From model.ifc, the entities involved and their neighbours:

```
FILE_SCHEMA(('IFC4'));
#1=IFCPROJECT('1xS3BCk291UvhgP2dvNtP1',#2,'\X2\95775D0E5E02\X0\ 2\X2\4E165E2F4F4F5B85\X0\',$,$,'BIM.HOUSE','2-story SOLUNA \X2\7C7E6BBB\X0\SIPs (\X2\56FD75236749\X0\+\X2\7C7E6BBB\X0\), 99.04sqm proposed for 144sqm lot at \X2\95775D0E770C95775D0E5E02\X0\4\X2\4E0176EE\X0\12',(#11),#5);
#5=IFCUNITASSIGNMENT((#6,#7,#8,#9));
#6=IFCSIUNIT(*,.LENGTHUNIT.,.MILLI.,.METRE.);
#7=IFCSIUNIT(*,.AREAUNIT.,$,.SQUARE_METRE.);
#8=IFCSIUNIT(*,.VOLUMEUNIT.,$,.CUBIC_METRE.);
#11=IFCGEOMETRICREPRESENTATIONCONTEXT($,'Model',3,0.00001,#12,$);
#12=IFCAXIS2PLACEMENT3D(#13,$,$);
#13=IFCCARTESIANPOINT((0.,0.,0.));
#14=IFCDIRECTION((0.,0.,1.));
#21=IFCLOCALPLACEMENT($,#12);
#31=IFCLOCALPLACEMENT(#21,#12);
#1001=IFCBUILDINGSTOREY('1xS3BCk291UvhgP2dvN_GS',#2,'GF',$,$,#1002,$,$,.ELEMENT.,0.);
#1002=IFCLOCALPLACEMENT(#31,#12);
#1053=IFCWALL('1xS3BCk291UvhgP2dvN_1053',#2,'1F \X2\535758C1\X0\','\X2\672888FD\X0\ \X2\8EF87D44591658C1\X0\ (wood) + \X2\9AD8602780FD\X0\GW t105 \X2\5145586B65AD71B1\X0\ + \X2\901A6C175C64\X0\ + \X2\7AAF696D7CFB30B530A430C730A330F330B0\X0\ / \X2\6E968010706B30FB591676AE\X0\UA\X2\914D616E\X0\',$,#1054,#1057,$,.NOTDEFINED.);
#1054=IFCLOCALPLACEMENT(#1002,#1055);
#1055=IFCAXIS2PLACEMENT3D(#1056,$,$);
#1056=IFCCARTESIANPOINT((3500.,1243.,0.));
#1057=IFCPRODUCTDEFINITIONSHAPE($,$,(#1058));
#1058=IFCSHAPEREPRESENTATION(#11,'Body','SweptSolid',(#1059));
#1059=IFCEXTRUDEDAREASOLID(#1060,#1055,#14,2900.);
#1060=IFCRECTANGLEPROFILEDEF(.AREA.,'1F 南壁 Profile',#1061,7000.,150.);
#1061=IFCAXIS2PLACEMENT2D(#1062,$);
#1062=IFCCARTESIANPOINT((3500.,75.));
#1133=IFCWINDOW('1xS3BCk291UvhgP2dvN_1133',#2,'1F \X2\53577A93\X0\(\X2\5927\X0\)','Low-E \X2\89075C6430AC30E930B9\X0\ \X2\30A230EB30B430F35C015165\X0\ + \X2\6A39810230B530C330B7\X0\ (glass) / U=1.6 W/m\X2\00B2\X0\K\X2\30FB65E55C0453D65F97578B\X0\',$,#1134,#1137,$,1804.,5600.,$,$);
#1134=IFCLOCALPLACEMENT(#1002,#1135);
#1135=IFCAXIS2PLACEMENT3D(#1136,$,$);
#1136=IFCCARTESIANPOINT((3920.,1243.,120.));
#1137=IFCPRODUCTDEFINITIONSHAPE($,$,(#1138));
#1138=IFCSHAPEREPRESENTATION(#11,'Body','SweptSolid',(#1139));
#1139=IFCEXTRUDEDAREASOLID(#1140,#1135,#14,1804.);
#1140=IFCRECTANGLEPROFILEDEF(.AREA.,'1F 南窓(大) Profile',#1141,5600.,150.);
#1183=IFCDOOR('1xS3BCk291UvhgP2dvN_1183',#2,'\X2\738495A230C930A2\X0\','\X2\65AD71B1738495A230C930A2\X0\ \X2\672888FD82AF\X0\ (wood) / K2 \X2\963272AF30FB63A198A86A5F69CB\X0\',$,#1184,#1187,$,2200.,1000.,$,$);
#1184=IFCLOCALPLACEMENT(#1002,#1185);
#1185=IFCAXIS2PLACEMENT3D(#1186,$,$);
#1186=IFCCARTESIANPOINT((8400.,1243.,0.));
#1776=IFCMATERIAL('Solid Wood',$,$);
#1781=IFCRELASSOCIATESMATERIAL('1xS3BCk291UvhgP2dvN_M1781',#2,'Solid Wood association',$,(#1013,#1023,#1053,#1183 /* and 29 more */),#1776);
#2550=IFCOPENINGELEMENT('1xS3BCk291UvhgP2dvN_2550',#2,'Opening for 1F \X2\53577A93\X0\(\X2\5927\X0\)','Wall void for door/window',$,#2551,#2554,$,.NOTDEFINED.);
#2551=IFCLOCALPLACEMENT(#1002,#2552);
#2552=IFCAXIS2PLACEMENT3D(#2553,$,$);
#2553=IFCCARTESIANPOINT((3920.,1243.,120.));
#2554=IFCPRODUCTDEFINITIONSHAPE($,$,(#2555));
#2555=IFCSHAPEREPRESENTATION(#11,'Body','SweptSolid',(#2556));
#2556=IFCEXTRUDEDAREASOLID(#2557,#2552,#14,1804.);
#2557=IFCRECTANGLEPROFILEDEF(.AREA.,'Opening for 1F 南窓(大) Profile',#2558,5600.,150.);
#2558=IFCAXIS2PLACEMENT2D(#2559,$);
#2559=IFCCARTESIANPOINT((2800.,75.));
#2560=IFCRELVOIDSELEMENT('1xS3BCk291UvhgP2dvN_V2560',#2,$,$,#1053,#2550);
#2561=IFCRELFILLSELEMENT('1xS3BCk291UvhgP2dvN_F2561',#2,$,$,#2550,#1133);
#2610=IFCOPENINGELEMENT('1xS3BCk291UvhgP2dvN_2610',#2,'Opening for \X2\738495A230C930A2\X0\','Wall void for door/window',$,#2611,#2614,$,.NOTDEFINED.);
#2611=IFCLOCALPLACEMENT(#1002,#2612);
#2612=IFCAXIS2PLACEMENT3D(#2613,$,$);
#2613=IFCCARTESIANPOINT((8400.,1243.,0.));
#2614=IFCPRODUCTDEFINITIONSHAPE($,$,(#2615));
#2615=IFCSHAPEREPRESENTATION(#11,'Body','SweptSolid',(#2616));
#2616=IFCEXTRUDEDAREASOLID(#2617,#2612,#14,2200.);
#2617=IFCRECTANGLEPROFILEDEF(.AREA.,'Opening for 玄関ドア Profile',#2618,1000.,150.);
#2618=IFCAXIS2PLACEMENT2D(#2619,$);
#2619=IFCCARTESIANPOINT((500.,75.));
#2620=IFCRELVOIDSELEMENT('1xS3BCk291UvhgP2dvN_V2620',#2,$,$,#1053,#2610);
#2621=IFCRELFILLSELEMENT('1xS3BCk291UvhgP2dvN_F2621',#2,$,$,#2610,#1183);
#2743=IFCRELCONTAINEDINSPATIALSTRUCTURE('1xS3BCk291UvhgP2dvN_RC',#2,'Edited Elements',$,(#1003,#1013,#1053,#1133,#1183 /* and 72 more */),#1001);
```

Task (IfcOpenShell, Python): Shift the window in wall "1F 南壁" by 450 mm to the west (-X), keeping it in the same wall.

```python
import ifcopenshell
import ifcopenshell.api.geometry
import ifcopenshell.util.placement
import ifcopenshell.util.unit

model = ifcopenshell.open("model.ifc")
unit_scale = ifcopenshell.util.unit.calculate_unit_scale(model)

window = model.by_guid("1xS3BCk291UvhgP2dvN_1133")
opening = window.FillsVoids[0].RelatingOpeningElement
wall = opening.VoidsElements[0].RelatingBuildingElement

wall_matrix = ifcopenshell.util.placement.get_local_placement(wall.ObjectPlacement)
shift = wall_matrix[:3, 0] * -0.45 / unit_scale
before = ifcopenshell.util.placement.get_local_placement(window.ObjectPlacement)[:3, 3].copy()

# The window is not placed relative to its opening, so move both.
for product in (opening, window):
    matrix = ifcopenshell.util.placement.get_local_placement(product.ObjectPlacement)
    matrix[:3, 3] += shift
    ifcopenshell.api.geometry.edit_object_placement(model, product=product, matrix=matrix, is_si=False)

after = ifcopenshell.util.placement.get_local_placement(window.ObjectPlacement)[:3, 3]
print("window moved by", (after - before).round(3) + 0.0)

model.write("model_v2.ifc")
```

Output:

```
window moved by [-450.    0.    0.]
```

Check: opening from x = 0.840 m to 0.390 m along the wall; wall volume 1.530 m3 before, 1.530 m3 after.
